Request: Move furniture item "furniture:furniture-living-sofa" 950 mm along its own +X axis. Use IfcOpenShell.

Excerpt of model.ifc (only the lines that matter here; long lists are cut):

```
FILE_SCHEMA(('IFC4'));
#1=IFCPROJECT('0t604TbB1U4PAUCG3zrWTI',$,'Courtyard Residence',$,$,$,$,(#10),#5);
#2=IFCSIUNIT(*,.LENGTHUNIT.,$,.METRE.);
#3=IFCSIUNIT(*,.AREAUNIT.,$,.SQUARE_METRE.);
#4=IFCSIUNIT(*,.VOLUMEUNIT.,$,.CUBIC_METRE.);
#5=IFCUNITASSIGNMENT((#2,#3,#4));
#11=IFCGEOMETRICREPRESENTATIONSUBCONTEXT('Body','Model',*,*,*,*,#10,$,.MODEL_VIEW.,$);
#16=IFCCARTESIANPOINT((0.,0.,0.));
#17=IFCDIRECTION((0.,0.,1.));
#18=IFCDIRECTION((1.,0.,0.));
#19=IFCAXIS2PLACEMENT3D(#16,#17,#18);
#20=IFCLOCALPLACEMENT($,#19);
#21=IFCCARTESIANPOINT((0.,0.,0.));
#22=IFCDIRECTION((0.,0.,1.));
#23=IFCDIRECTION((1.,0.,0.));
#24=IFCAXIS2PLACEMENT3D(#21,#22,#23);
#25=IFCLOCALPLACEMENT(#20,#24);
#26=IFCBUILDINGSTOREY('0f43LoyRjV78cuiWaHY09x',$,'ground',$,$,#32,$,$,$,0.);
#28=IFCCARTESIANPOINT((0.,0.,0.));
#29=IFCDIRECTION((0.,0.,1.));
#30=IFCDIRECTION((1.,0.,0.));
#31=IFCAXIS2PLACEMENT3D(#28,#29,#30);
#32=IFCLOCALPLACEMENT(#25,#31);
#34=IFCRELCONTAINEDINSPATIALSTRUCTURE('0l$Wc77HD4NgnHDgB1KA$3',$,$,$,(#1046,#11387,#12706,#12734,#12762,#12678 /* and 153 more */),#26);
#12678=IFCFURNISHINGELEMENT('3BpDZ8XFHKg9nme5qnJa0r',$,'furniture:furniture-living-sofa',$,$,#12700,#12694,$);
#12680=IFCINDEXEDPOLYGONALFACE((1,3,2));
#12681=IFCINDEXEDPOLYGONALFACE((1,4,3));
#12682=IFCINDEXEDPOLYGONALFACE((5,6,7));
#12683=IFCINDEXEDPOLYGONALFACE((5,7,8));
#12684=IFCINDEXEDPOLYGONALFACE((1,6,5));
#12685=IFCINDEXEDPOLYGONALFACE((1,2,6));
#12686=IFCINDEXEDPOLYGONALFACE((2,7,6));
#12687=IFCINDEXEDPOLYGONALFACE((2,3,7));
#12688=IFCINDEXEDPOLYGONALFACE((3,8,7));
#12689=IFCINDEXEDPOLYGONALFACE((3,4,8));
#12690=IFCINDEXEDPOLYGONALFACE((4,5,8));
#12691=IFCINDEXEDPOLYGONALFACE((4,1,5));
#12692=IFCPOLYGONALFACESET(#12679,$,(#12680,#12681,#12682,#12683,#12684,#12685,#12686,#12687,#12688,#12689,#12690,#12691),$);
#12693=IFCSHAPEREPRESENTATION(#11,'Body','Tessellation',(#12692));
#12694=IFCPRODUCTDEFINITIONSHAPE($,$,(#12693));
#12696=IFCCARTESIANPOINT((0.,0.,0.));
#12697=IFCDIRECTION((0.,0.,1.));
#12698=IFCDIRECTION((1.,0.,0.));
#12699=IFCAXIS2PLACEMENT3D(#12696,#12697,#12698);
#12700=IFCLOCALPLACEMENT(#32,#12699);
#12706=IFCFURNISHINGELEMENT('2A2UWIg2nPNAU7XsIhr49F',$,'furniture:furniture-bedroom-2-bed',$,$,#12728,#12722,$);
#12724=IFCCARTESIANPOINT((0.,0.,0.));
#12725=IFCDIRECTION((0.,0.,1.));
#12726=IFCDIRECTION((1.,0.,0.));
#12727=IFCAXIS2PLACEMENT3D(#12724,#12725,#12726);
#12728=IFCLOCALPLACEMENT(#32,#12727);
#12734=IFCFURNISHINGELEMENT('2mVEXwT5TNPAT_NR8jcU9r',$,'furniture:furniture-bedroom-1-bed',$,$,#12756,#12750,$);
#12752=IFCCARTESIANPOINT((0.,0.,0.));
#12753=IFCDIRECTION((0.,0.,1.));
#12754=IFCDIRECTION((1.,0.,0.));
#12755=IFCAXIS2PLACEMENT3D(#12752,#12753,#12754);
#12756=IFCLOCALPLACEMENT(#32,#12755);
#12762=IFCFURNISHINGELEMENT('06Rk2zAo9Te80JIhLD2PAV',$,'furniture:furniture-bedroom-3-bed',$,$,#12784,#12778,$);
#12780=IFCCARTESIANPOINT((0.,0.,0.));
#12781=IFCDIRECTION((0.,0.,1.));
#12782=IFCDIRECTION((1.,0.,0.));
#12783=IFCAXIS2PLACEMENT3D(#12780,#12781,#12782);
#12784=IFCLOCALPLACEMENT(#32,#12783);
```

```python
import ifcopenshell
import ifcopenshell.api.geometry
import ifcopenshell.util.placement

model = ifcopenshell.open("model.ifc")

item = model.by_guid("3BpDZ8XFHKg9nme5qnJa0r")
matrix = ifcopenshell.util.placement.get_local_placement(item.ObjectPlacement)
matrix[:3, 3] += matrix[:3, 0] * 0.95
ifcopenshell.api.geometry.edit_object_placement(model, product=item, matrix=matrix, is_si=False)

print(ifcopenshell.util.placement.get_local_placement(item.ObjectPlacement).round(3) + 0.0)

model.write("model_rev.ifc")
```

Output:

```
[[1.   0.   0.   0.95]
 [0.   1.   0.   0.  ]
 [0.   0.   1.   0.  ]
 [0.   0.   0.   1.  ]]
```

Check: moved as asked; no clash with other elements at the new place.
